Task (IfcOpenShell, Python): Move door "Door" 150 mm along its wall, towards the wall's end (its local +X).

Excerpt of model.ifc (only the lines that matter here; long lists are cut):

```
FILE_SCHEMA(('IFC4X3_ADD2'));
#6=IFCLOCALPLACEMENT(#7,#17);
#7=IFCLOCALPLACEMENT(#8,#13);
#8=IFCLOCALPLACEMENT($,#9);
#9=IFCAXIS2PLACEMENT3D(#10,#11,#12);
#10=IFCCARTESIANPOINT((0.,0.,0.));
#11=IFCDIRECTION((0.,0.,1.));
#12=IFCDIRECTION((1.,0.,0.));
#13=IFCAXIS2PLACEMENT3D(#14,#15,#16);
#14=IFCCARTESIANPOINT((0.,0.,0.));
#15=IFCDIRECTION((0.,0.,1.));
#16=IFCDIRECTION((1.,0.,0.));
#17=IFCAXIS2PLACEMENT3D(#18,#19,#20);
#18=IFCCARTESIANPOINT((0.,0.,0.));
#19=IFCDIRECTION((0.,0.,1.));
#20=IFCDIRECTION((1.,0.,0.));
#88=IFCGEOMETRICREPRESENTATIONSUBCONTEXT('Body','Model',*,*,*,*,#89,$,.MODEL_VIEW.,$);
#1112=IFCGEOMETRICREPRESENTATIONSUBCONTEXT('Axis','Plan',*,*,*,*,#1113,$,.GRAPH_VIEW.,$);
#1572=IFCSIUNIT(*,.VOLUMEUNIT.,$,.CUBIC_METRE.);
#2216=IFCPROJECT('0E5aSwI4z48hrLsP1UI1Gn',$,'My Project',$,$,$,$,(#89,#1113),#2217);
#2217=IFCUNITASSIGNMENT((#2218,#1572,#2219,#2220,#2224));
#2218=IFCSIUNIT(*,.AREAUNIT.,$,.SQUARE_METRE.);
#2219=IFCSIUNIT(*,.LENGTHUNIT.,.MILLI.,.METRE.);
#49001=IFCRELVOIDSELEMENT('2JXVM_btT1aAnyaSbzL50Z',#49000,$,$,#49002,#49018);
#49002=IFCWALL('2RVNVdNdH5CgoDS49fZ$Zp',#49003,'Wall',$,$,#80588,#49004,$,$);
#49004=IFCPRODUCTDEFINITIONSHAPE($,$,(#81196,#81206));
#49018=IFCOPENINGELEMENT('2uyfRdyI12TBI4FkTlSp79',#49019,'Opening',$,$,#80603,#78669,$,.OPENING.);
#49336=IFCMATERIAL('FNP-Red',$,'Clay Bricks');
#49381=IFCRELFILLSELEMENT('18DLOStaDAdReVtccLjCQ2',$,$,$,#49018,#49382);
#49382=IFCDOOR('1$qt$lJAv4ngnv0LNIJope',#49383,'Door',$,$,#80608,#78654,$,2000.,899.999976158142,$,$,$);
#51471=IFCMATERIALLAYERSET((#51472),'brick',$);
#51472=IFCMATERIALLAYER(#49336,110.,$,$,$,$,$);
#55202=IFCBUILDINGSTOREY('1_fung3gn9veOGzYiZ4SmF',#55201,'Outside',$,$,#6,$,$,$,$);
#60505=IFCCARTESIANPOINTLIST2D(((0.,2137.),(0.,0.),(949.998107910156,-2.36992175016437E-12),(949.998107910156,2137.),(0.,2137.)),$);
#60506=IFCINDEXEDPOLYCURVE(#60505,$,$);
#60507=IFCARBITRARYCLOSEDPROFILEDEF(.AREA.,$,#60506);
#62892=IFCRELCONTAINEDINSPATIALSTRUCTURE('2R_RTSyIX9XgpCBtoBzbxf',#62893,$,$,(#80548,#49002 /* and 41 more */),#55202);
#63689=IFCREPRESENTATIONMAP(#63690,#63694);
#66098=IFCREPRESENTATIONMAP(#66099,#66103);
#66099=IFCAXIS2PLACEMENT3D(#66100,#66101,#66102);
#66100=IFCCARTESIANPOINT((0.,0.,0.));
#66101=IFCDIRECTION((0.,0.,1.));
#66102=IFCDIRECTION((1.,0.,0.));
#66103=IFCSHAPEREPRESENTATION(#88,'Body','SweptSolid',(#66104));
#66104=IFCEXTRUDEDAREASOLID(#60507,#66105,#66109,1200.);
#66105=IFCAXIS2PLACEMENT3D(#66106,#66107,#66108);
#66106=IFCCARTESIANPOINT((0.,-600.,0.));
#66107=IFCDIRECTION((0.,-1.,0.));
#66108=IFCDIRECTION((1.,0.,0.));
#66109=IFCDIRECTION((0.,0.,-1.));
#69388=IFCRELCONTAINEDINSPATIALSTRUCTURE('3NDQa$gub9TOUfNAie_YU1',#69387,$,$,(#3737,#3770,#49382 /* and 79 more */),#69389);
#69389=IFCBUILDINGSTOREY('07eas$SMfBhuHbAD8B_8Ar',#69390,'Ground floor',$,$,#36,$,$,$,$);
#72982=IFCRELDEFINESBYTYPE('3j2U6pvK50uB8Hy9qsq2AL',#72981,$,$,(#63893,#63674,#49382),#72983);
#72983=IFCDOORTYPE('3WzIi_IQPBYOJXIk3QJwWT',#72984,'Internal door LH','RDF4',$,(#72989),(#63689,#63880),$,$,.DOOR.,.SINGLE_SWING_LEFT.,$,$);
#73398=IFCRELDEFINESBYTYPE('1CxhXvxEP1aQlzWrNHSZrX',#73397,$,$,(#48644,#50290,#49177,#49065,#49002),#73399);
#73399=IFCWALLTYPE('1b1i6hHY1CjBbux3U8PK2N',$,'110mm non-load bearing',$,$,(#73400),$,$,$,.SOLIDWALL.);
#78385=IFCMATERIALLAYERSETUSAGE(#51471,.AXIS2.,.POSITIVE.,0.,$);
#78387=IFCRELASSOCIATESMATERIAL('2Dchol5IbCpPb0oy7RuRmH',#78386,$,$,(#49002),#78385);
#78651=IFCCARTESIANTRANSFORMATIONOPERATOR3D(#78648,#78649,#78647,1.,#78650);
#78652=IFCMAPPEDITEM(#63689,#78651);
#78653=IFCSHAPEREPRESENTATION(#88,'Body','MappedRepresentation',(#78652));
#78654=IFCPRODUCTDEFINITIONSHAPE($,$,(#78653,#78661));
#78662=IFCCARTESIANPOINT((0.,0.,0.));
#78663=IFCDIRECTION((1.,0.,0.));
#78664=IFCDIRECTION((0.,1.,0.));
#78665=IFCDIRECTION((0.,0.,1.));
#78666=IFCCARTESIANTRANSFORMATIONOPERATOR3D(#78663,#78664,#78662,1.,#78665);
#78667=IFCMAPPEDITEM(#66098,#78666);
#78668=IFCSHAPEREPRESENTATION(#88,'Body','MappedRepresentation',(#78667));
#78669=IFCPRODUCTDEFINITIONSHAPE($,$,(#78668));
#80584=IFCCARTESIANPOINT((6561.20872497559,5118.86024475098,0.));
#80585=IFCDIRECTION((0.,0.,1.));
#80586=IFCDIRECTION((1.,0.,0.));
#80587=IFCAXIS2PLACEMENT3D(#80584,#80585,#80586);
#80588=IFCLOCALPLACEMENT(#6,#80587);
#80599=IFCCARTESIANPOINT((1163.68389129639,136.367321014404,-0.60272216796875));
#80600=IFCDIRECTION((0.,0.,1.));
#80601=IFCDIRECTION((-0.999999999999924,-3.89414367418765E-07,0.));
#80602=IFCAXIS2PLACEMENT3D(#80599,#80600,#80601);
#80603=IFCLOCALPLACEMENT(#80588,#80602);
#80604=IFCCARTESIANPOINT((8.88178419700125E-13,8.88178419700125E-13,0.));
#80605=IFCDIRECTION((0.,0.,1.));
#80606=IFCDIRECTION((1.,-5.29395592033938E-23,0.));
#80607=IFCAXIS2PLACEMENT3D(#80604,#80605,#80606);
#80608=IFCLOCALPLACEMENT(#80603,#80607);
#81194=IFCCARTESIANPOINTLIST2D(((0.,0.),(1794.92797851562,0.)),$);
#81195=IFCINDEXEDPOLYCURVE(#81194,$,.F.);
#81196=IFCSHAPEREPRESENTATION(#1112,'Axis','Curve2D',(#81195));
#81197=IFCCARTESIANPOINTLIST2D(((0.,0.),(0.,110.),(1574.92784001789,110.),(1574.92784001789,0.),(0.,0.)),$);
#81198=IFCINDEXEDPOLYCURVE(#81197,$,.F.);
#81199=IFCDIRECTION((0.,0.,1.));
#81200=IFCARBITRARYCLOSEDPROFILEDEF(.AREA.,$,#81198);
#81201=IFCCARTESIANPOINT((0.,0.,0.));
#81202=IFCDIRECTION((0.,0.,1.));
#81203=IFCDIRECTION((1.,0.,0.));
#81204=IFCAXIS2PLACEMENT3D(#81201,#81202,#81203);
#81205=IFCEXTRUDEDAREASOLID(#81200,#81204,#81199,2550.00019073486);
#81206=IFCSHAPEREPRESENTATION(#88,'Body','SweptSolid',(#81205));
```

```python
import ifcopenshell
import ifcopenshell.api.geometry
import ifcopenshell.util.placement

model = ifcopenshell.open("model.ifc")

door = model.by_guid("1$qt$lJAv4ngnv0LNIJope")
opening = door.FillsVoids[0].RelatingOpeningElement
wall = opening.VoidsElements[0].RelatingBuildingElement

wall_matrix = ifcopenshell.util.placement.get_local_placement(wall.ObjectPlacement)
shift = wall_matrix[:3, 0] * 150.0
before = ifcopenshell.util.placement.get_local_placement(door.ObjectPlacement)[:3, 3].copy()

# The door is placed relative to its opening, so it follows when the opening moves.
matrix = ifcopenshell.util.placement.get_local_placement(opening.ObjectPlacement)
matrix[:3, 3] += shift
ifcopenshell.api.geometry.edit_object_placement(
    model, product=opening, matrix=matrix, is_si=False, should_transform_children=True
)

after = ifcopenshell.util.placement.get_local_placement(door.ObjectPlacement)[:3, 3]
print("door moved by", (after - before).round(3) + 0.0)

model.write("model-out.ifc")
```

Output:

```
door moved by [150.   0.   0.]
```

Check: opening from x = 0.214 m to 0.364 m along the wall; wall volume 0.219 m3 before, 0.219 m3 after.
